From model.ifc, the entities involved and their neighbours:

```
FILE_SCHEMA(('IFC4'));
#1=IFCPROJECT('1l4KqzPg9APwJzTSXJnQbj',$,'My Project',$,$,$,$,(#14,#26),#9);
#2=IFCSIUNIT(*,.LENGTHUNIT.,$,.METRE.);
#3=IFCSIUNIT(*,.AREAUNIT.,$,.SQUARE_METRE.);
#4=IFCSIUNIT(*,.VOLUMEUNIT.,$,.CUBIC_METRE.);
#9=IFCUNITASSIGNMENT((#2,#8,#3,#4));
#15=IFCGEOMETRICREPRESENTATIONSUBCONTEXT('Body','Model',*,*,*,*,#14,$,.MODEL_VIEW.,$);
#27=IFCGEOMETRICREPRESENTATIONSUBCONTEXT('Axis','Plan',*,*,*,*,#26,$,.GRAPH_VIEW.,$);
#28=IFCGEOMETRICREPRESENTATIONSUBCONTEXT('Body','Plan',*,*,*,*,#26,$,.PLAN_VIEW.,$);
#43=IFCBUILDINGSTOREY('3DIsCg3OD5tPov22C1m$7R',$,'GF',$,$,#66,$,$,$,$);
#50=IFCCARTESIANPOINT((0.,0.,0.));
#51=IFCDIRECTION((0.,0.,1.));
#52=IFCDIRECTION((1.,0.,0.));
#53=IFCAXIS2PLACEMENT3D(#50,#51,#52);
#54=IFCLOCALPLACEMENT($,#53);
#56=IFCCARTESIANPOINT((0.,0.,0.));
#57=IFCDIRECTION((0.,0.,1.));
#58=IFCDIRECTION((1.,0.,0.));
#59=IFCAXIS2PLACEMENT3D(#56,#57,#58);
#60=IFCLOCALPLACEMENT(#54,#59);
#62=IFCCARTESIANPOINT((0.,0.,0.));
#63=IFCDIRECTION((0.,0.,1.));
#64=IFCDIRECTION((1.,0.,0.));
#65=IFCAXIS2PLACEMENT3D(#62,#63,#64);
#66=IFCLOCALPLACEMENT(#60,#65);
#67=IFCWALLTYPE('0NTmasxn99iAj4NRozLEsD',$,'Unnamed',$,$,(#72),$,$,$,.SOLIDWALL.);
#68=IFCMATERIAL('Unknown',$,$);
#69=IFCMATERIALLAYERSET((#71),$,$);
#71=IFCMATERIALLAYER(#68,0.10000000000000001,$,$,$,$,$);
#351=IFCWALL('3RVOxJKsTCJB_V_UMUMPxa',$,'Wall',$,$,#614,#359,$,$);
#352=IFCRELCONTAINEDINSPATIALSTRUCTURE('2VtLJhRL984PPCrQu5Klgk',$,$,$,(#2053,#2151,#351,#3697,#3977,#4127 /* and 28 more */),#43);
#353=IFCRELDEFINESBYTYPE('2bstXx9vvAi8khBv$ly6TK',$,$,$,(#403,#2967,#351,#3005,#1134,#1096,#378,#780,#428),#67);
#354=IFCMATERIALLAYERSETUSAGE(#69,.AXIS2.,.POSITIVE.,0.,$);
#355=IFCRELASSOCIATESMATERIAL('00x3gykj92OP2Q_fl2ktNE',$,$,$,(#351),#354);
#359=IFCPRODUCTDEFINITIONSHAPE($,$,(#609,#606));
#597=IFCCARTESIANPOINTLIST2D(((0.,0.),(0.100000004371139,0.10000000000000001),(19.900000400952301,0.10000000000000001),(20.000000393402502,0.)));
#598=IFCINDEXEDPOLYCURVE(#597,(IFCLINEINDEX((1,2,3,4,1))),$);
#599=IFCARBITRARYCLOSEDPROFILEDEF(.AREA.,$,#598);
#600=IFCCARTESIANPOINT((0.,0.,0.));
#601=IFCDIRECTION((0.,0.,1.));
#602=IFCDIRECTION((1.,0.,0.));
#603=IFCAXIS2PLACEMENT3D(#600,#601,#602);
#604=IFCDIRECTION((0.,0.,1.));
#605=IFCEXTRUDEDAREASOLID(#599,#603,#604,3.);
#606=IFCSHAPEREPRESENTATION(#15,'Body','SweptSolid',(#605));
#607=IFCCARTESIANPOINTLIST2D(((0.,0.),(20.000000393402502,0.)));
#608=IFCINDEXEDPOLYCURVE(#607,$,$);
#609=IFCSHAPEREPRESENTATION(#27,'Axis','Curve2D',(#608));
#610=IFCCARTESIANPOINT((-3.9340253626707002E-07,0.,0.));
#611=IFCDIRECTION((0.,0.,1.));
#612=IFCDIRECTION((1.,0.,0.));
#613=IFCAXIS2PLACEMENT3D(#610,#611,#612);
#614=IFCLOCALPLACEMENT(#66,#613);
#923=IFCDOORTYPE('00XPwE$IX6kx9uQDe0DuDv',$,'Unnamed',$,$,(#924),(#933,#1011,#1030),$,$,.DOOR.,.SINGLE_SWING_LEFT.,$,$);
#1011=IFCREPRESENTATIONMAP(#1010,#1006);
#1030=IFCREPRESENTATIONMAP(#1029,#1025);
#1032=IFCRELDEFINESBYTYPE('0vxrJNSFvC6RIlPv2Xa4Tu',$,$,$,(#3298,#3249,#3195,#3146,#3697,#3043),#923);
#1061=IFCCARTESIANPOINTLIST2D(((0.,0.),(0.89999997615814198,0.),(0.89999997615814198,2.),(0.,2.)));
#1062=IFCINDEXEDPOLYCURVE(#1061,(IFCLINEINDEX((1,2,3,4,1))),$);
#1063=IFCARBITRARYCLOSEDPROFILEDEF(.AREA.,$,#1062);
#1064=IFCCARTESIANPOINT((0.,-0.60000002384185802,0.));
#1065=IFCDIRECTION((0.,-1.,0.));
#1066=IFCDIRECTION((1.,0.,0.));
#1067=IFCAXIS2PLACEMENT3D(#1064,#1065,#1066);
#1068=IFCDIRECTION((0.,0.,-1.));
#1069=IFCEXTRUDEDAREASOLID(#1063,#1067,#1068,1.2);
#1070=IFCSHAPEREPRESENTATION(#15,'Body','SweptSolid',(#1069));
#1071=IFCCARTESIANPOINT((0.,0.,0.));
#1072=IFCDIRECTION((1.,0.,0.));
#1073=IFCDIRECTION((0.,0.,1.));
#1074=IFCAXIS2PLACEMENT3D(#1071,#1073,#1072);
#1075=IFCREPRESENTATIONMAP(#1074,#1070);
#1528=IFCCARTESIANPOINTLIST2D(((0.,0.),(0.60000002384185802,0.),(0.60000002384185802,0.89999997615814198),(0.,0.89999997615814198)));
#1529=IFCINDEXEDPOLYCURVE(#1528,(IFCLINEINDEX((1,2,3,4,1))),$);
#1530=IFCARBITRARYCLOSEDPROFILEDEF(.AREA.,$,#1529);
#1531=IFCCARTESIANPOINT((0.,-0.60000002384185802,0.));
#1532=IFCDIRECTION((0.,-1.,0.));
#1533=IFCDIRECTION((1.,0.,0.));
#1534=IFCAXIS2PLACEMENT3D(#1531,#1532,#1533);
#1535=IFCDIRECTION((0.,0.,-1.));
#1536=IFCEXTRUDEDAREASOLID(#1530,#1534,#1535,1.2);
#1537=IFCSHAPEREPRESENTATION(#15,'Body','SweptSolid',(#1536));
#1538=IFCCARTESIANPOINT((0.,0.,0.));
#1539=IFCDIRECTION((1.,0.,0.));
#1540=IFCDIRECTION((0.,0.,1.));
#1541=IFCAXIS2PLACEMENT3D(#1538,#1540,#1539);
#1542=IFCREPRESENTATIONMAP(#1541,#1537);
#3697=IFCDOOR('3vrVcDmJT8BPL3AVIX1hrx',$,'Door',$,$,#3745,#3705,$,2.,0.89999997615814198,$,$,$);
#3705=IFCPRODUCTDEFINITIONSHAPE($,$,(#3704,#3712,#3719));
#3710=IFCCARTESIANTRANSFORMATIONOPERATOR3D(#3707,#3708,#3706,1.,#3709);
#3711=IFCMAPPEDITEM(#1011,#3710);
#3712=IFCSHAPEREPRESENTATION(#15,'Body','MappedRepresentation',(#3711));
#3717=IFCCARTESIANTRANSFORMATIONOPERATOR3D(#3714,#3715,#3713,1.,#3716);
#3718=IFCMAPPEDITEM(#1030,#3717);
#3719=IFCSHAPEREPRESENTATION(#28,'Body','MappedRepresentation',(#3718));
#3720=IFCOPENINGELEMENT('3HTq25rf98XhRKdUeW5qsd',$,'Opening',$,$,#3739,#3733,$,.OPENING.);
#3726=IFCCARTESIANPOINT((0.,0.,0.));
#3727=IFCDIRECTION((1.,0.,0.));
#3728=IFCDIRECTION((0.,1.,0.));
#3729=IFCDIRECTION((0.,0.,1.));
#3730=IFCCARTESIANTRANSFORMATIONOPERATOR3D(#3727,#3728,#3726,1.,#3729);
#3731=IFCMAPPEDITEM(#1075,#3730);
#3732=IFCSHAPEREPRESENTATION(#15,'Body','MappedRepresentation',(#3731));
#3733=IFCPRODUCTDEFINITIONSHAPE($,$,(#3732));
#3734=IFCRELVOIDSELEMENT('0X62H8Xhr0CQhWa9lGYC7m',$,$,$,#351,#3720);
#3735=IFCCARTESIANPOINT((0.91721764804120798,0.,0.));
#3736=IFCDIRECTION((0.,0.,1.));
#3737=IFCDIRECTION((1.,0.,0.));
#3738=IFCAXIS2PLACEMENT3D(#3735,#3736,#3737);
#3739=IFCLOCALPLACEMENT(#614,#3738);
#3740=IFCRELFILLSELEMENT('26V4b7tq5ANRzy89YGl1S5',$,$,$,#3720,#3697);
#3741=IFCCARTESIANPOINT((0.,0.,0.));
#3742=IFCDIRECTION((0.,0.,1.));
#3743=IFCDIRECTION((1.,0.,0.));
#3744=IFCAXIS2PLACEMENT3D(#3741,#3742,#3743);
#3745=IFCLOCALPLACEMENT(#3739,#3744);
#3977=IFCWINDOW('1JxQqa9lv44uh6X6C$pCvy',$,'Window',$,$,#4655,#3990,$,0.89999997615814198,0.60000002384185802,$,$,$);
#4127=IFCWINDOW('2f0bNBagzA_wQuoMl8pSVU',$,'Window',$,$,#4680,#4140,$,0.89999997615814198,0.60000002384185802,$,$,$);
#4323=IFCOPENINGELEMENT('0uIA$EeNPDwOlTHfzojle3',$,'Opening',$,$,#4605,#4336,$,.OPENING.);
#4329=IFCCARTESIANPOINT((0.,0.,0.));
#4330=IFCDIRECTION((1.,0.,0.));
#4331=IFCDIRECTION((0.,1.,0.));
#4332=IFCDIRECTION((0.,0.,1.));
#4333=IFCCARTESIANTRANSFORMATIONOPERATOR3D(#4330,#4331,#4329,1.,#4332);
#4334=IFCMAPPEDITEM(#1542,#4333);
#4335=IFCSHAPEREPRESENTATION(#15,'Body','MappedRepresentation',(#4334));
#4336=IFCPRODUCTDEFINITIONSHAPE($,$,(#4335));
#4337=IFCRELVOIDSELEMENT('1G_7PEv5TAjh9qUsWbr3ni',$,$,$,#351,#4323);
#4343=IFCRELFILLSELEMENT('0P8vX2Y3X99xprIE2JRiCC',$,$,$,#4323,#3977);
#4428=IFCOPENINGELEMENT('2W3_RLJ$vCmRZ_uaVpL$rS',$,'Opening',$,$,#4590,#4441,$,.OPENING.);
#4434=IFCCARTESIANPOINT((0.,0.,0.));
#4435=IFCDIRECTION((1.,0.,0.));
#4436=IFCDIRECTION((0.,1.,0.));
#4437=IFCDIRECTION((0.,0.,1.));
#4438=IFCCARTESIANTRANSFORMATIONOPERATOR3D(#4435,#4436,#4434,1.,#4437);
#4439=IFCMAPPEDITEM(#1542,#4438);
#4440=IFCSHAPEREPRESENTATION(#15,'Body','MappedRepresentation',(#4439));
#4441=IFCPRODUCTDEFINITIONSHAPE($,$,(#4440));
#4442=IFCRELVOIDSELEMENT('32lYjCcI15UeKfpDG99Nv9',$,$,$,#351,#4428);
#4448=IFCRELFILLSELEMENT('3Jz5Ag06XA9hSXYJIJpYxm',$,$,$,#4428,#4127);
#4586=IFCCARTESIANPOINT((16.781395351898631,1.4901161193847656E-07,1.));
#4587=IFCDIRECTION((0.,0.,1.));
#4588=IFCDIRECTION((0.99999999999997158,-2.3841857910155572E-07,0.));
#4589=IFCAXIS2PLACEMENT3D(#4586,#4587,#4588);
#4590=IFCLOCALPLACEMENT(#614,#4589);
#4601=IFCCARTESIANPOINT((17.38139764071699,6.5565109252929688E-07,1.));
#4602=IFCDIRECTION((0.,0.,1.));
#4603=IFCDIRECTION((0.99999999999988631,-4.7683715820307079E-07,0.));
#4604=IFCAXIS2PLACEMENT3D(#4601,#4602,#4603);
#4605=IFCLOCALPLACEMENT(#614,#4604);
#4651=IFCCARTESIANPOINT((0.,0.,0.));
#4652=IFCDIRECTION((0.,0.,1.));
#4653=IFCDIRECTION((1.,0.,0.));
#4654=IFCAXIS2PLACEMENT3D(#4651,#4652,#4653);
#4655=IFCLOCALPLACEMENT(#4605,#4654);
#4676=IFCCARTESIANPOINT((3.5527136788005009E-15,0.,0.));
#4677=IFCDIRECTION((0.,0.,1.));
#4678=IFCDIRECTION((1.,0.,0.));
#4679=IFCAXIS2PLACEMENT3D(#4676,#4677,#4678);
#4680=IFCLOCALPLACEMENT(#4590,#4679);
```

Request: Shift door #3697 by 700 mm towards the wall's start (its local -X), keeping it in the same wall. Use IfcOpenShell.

```python
import ifcopenshell
import ifcopenshell.api.geometry
import ifcopenshell.util.placement
import ifcopenshell.util.unit

model = ifcopenshell.open("model.ifc")
unit_scale = ifcopenshell.util.unit.calculate_unit_scale(model)

door = model.by_guid("3vrVcDmJT8BPL3AVIX1hrx")
opening = door.FillsVoids[0].RelatingOpeningElement
wall = opening.VoidsElements[0].RelatingBuildingElement

wall_matrix = ifcopenshell.util.placement.get_local_placement(wall.ObjectPlacement)
shift = wall_matrix[:3, 0] * -0.7 / unit_scale
before = ifcopenshell.util.placement.get_local_placement(door.ObjectPlacement)[:3, 3].copy()

# The door is placed relative to its opening, so it follows when the opening moves.
matrix = ifcopenshell.util.placement.get_local_placement(opening.ObjectPlacement)
matrix[:3, 3] += shift
ifcopenshell.api.geometry.edit_object_placement(
    model, product=opening, matrix=matrix, is_si=False, should_transform_children=True
)

after = ifcopenshell.util.placement.get_local_placement(door.ObjectPlacement)[:3, 3]
print("door moved by", (after - before).round(3) + 0.0)

model.write("model_rev.ifc")
```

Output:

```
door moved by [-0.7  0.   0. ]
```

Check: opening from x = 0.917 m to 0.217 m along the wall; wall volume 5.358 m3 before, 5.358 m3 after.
